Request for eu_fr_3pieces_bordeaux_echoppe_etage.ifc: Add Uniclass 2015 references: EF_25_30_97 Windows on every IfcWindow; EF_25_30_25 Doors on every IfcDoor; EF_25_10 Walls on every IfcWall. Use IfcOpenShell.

First a look at what the model holds.

```python
import ifcopenshell

model = ifcopenshell.open("eu_fr_3pieces_bordeaux_echoppe_etage.ifc")
print(model.schema)
print("classifications:", [c.Name for c in model.by_type("IfcClassification")])
for ifc_class in ("IfcDoor", "IfcRoof", "IfcStair", "IfcWall", "IfcWindow"):
    print(ifc_class, len(model.by_type(ifc_class)))
```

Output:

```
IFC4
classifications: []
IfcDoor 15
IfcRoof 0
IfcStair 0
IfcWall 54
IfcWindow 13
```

```python
import ifcopenshell
import ifcopenshell.api.classification

model = ifcopenshell.open("eu_fr_3pieces_bordeaux_echoppe_etage.ifc")

system = ifcopenshell.api.classification.add_classification(model, classification="Uniclass 2015")

codes = {
    "IfcWindow": ("EF_25_30_97", "Windows"),
    "IfcDoor": ("EF_25_30_25", "Doors"),
    "IfcWall": ("EF_25_10", "Walls"),
}
for ifc_class, (code, name) in codes.items():
    products = model.by_type(ifc_class)
    ifcopenshell.api.classification.add_reference(
        model, products=products, classification=system, identification=code, name=name
    )
    print(code, len(products))

model.write("eu_fr_3pieces_bordeaux_echoppe_etage_edited.ifc")
```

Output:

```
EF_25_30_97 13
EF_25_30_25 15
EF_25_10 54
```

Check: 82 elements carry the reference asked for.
